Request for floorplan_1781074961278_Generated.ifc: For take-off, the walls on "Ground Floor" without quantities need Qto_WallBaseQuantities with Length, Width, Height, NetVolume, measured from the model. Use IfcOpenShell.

First a look at what the model holds.

```python
import ifcopenshell
import ifcopenshell.util.element
import ifcopenshell.util.unit

model = ifcopenshell.open("floorplan_1781074961278_Generated.ifc")
print(model.schema)
for unit_type in ("LENGTHUNIT", "AREAUNIT", "VOLUMEUNIT"):
    print(unit_type, ifcopenshell.util.unit.calculate_unit_scale(model, unit_type))
storey = next(s for s in model.by_type("IfcBuildingStorey") if s.Name == "Ground Floor")
walls = [e for e in ifcopenshell.util.element.get_decomposition(storey) if e.is_a("IfcWall")]
for e in sorted(walls, key=lambda e: e.id()):
    print(e.id(), e.is_a(), e.Name, list(ifcopenshell.util.element.get_psets(e, qtos_only=True)), sep=" | ")
```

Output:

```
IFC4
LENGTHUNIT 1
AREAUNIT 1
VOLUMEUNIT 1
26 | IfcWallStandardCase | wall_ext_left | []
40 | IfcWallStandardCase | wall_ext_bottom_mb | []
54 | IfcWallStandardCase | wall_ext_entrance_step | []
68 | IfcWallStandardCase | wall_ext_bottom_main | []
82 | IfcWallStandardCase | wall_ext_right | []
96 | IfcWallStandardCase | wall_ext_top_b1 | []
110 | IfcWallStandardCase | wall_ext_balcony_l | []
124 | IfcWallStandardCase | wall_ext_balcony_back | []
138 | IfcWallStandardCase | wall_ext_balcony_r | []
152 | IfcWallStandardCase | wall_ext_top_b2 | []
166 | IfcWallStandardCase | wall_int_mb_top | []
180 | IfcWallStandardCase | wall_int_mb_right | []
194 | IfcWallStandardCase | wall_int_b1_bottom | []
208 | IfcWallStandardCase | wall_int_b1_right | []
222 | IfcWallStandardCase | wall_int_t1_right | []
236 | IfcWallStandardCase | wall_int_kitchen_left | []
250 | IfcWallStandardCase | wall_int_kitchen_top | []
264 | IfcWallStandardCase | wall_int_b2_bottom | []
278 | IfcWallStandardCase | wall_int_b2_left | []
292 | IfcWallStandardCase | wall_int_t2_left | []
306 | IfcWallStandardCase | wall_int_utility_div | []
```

```python
import ifcopenshell
import ifcopenshell.api.pset
import ifcopenshell.geom
import ifcopenshell.util.element
import ifcopenshell.util.shape
import ifcopenshell.util.unit

model = ifcopenshell.open("floorplan_1781074961278_Generated.ifc")
unit_scale = ifcopenshell.util.unit.calculate_unit_scale(model)
volume_scale = ifcopenshell.util.unit.calculate_unit_scale(model, "VOLUMEUNIT")
settings = ifcopenshell.geom.settings()

storey = next(s for s in model.by_type("IfcBuildingStorey") if s.Name == "Ground Floor")
walls = [e for e in ifcopenshell.util.element.get_decomposition(storey) if e.is_a("IfcWall")]

for e in sorted(walls, key=lambda e: e.id()):
    if ifcopenshell.util.element.get_psets(e, qtos_only=True, should_inherit=False):
        continue
    # Geometry comes back in metres, in the element's own axes.
    shape = ifcopenshell.geom.create_shape(settings, e)
    values = {
        "Length": ifcopenshell.util.shape.get_x(shape.geometry) / unit_scale,
        "Width": ifcopenshell.util.shape.get_y(shape.geometry) / unit_scale,
        "Height": ifcopenshell.util.shape.get_z(shape.geometry) / unit_scale,
        "NetVolume": ifcopenshell.util.shape.get_volume(shape.geometry) / volume_scale,
    }
    qto = ifcopenshell.api.pset.add_qto(model, product=e, name="Qto_WallBaseQuantities")
    ifcopenshell.api.pset.edit_qto(model, qto=qto, properties=values)
    print(e.id(), {k: round(v, 3) for k, v in values.items()})

model.write("floorplan_1781074961278_Generated_v2.ifc")
```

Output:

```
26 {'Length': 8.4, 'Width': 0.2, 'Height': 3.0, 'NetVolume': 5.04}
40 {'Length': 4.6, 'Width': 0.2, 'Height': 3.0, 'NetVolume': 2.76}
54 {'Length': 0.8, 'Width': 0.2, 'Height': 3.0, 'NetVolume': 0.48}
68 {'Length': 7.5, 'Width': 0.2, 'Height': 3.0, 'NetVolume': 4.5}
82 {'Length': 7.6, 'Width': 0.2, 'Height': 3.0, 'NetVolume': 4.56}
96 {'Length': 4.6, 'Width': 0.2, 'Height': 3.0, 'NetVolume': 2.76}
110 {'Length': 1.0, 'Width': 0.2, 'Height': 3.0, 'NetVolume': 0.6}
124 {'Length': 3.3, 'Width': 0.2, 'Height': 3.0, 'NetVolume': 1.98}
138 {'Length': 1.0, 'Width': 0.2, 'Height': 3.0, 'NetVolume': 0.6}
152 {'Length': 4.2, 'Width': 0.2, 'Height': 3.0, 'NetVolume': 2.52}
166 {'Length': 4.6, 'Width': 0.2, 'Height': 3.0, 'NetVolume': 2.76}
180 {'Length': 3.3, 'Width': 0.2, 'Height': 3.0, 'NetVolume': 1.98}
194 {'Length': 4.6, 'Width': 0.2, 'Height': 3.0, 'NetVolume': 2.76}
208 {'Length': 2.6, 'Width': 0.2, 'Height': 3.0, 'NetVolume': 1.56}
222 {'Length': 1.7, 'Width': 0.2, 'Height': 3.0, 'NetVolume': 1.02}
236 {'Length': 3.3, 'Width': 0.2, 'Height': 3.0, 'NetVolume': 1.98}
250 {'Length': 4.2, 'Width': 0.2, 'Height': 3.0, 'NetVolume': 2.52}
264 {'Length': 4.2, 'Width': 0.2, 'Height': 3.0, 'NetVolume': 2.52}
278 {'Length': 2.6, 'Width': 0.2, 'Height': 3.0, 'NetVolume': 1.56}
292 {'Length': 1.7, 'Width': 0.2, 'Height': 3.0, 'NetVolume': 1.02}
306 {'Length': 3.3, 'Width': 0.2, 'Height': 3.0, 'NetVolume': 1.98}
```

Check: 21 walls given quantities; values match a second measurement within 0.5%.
